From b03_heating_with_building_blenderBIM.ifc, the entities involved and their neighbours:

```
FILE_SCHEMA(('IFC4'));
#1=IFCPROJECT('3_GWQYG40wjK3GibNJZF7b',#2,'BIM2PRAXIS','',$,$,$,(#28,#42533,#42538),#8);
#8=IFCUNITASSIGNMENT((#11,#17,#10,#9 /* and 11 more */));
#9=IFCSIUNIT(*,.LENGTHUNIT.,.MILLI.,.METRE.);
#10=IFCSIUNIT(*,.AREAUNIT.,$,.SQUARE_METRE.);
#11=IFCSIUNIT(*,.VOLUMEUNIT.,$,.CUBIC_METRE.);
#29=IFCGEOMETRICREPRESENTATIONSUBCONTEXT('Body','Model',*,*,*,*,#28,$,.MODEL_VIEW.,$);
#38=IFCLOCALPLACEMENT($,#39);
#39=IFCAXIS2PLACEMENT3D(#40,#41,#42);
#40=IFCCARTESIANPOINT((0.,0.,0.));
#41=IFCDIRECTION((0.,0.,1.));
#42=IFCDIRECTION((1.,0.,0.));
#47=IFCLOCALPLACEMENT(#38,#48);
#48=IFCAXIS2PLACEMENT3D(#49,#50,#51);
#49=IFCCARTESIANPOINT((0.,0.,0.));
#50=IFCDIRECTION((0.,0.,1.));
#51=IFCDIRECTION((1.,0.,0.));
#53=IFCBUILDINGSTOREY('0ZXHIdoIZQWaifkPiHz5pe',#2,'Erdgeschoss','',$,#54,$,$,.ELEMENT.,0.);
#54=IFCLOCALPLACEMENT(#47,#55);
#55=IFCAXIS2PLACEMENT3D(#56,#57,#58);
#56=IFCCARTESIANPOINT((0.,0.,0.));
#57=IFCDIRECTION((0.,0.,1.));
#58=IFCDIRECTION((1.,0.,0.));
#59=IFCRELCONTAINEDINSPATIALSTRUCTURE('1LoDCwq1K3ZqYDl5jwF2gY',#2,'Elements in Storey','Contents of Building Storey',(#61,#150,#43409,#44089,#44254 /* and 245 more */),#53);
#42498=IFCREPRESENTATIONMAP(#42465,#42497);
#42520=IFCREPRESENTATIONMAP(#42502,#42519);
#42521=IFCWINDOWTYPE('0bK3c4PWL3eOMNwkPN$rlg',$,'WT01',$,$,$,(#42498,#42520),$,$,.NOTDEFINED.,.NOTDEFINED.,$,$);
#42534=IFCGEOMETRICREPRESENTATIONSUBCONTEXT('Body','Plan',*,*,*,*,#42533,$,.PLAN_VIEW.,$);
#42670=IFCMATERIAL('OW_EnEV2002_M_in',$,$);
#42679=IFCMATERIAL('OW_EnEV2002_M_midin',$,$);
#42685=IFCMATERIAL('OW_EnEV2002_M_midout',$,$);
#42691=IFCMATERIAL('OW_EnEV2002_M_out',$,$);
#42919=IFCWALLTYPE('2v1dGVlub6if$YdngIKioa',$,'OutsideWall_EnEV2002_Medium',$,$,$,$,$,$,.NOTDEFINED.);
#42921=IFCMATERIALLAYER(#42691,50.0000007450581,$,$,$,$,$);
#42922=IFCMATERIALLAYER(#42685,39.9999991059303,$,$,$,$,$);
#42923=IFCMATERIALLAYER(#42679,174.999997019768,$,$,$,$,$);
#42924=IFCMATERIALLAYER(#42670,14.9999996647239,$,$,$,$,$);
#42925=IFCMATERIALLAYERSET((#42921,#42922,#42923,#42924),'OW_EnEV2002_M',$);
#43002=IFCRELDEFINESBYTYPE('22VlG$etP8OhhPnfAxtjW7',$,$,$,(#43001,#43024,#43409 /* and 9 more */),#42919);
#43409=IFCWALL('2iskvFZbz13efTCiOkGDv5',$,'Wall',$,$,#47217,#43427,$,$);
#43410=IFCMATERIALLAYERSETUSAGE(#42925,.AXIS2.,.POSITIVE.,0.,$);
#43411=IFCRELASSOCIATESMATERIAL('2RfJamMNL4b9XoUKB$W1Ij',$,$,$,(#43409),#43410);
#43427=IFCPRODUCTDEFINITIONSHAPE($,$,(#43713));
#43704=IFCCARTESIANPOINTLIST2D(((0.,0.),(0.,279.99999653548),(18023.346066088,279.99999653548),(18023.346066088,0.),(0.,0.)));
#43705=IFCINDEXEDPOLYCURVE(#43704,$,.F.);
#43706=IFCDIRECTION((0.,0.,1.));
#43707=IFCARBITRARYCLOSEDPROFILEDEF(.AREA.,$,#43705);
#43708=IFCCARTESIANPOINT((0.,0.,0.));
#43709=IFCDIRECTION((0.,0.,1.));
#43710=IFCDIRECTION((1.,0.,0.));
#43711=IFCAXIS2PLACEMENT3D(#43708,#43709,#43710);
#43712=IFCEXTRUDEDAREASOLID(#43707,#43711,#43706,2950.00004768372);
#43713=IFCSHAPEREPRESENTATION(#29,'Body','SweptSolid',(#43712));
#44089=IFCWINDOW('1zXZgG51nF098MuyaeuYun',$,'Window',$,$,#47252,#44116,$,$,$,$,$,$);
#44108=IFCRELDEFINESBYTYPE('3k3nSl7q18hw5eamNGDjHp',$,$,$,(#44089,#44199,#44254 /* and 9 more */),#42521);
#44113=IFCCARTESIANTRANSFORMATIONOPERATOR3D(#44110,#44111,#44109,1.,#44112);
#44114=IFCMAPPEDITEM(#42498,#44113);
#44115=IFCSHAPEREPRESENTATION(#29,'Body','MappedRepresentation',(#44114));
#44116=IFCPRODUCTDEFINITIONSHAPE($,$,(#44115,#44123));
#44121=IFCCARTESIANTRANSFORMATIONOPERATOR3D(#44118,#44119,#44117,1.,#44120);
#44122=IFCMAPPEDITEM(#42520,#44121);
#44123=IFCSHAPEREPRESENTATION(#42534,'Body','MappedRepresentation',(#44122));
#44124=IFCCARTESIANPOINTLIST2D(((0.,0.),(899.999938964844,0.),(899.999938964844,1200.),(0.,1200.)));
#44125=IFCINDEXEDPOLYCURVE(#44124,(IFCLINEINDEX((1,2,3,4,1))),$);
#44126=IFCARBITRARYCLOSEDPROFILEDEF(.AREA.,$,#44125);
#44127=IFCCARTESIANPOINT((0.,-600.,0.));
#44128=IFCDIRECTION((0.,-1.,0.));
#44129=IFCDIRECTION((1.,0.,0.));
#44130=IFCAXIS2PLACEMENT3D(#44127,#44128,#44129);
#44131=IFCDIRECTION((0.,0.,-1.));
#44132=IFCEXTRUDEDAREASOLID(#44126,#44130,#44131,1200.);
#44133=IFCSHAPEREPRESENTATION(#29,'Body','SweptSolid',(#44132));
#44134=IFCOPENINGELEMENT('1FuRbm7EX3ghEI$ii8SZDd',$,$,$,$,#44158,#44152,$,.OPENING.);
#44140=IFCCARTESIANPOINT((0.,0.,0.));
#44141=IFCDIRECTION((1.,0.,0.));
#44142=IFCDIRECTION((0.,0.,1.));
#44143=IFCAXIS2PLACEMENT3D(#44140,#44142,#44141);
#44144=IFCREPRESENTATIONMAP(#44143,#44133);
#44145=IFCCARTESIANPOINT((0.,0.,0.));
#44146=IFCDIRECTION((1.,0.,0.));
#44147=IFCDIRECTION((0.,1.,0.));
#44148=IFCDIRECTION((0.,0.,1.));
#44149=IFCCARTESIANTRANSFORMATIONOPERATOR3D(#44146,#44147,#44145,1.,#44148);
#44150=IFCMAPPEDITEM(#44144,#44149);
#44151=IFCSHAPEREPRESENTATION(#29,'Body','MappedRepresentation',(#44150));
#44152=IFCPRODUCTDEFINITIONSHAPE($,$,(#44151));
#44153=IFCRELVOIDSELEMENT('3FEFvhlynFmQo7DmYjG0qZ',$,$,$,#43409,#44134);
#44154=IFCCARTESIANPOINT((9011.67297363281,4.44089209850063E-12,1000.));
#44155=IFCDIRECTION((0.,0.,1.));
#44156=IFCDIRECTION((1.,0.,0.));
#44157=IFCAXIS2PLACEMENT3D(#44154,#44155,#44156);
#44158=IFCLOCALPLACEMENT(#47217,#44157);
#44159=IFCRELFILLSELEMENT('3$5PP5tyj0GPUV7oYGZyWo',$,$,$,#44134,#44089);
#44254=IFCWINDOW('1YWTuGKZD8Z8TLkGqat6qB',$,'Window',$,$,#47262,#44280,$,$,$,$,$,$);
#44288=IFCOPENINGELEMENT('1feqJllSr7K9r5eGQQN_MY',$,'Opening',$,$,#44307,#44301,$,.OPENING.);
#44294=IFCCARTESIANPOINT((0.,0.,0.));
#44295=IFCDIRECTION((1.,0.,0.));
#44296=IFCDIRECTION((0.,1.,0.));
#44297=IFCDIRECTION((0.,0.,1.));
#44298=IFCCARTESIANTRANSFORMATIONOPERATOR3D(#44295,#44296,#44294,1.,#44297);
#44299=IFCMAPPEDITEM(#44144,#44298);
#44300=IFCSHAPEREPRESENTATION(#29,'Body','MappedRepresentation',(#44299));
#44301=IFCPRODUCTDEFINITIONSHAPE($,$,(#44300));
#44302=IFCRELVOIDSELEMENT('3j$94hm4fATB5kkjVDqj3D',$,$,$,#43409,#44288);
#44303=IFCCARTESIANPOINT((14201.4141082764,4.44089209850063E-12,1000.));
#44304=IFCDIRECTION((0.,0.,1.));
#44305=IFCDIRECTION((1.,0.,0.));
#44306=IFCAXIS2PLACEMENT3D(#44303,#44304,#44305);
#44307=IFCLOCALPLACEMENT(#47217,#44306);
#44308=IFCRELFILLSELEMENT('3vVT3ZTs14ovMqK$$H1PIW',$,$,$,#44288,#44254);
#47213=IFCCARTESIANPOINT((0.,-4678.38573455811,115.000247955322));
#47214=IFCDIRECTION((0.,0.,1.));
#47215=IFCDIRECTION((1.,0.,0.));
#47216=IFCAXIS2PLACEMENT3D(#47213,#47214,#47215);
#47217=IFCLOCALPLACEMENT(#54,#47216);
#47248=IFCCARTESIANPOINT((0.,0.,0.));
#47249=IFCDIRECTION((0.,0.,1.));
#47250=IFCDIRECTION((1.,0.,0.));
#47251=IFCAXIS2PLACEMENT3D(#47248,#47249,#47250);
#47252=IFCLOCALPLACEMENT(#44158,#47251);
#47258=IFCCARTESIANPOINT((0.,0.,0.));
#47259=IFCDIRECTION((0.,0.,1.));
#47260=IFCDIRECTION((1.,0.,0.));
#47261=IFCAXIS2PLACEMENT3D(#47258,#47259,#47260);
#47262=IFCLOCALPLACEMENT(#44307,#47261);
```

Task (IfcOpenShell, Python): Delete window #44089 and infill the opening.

```python
import ifcopenshell
import ifcopenshell.api.feature
import ifcopenshell.api.root
import ifcopenshell.geom
import ifcopenshell.util.shape

model = ifcopenshell.open("b03_heating_with_building_blenderBIM.ifc")
settings = ifcopenshell.geom.settings()


def volume(element):
    """Net volume in cubic metres, openings subtracted."""
    shape = ifcopenshell.geom.create_shape(settings, element)
    return ifcopenshell.util.shape.get_volume(shape.geometry)


window = model.by_guid("1zXZgG51nF098MuyaeuYun")
opening = window.FillsVoids[0].RelatingOpeningElement
wall = opening.VoidsElements[0].RelatingBuildingElement
before = volume(wall)

ifcopenshell.api.root.remove_product(model, product=window)
ifcopenshell.api.feature.remove_feature(model, feature=opening)

after = volume(wall)

print(f"wall volume {before:.3f} -> {after:.3f} m3")

model.write("b03_heating_with_building_blenderBIM_updated.ifc")
```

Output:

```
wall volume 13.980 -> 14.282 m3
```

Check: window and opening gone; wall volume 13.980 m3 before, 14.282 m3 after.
